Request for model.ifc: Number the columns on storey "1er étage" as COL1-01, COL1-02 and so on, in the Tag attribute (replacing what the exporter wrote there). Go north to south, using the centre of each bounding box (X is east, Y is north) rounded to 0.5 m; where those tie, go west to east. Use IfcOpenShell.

First a look at what the model holds.

```python
import ifcopenshell
import ifcopenshell.util.element
import ifcopenshell.util.placement

model = ifcopenshell.open("model.ifc")
print(model.schema)
storey = next(s for s in model.by_type("IfcBuildingStorey") if s.Name == "1er étage")
columns = [e for e in ifcopenshell.util.element.get_decomposition(storey) if e.is_a("IfcColumn")]
for e in sorted(columns, key=lambda e: e.id()):
    origin = ifcopenshell.util.placement.get_local_placement(e.ObjectPlacement)[:3, 3]
    print(e.id(), e.Tag, e.Name, origin.round(2) + 0.0, sep=" | ")
```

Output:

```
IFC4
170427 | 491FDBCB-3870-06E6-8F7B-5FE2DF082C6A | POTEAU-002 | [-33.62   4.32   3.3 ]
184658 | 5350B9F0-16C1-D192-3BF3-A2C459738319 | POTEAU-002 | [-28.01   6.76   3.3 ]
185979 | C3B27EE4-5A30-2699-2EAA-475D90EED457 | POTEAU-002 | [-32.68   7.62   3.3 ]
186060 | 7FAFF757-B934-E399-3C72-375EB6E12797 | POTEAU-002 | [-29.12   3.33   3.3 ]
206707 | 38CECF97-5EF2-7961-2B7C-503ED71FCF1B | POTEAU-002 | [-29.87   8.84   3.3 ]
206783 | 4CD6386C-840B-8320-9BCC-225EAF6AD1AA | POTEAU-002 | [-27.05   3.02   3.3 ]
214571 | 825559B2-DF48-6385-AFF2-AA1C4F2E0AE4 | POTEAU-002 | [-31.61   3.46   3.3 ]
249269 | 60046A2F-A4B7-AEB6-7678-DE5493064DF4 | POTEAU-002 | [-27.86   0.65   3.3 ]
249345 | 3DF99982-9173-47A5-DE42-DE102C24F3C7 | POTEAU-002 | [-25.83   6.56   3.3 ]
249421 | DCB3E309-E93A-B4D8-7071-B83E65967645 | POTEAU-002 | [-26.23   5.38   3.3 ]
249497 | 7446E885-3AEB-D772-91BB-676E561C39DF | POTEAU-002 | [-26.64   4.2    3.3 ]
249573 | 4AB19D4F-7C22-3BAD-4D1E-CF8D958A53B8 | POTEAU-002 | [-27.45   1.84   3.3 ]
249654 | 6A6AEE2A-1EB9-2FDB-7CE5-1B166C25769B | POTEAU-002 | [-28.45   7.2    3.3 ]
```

```python
import ifcopenshell
import ifcopenshell.geom
import ifcopenshell.util.element
import ifcopenshell.util.shape

model = ifcopenshell.open("model.ifc")
settings = ifcopenshell.geom.settings()
settings.set("use-world-coords", True)


def centre(element):
    shape = ifcopenshell.geom.create_shape(settings, element)
    return ifcopenshell.util.shape.get_bbox_centroid(shape.geometry)


storey = next(s for s in model.by_type("IfcBuildingStorey") if s.Name == "1er étage")
columns = [e for e in ifcopenshell.util.element.get_decomposition(storey) if e.is_a("IfcColumn")]

# Insertion points can sit at a corner or the storey origin, so sort by the geometry (in metres).
centres = {e: centre(e) for e in columns}
columns.sort(key=lambda e: (-round(centres[e][1] / 0.5), centres[e][0]))

for i, e in enumerate(columns, start=1):
    number = f"COL1-{i:02d}"
    e.Tag = number
    print(e.id(), number)

model.write("model_edited.ifc")
```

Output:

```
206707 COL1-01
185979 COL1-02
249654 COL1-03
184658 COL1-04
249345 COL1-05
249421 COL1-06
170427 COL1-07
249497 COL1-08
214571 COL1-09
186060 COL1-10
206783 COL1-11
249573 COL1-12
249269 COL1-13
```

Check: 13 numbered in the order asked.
